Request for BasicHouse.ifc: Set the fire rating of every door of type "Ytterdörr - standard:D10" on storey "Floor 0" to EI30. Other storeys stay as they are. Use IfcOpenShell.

First a look at what the model holds.

```python
import ifcopenshell
import ifcopenshell.util.element

model = ifcopenshell.open("BasicHouse.ifc")
print(model.schema)
storey = next(s for s in model.by_type("IfcBuildingStorey") if s.Name == "Floor 0")
doors = [e for e in ifcopenshell.util.element.get_decomposition(storey) if e.is_a("IfcDoor")]
seen = {}
for e in doors:
    element_type = ifcopenshell.util.element.get_type(e)
    key = (element_type.Name if element_type != e and element_type else None, ifcopenshell.util.element.get_pset(e, "Pset_DoorCommon", "FireRating"))
    seen[key] = seen.get(key, 0) + 1
for (name, value), count in sorted(seen.items(), key=str):
    print(count, "x", name, "|", value)
```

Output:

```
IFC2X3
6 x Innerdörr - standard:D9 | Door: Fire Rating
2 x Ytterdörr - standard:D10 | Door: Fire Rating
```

```python
import ifcopenshell
import ifcopenshell.api.pset
import ifcopenshell.util.element

model = ifcopenshell.open("BasicHouse.ifc")

storey = next(s for s in model.by_type("IfcBuildingStorey") if s.Name == "Floor 0")
doors = [e for e in ifcopenshell.util.element.get_decomposition(storey) if e.is_a("IfcDoor")]

count = 0
for e in doors:
    element_type = ifcopenshell.util.element.get_type(e)
    if element_type in (None, e) or element_type.Name != "Ytterdörr - standard:D10":
        continue
    # add_pset returns the element's existing set when there is one.
    pset = ifcopenshell.api.pset.add_pset(model, product=e, name="Pset_DoorCommon")
    ifcopenshell.api.pset.edit_pset(model, pset=pset, properties={"FireRating": "EI30"})
    count += 1

print(count, "doors updated")

model.write("BasicHouse_v2.ifc")
```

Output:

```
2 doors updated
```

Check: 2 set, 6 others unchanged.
